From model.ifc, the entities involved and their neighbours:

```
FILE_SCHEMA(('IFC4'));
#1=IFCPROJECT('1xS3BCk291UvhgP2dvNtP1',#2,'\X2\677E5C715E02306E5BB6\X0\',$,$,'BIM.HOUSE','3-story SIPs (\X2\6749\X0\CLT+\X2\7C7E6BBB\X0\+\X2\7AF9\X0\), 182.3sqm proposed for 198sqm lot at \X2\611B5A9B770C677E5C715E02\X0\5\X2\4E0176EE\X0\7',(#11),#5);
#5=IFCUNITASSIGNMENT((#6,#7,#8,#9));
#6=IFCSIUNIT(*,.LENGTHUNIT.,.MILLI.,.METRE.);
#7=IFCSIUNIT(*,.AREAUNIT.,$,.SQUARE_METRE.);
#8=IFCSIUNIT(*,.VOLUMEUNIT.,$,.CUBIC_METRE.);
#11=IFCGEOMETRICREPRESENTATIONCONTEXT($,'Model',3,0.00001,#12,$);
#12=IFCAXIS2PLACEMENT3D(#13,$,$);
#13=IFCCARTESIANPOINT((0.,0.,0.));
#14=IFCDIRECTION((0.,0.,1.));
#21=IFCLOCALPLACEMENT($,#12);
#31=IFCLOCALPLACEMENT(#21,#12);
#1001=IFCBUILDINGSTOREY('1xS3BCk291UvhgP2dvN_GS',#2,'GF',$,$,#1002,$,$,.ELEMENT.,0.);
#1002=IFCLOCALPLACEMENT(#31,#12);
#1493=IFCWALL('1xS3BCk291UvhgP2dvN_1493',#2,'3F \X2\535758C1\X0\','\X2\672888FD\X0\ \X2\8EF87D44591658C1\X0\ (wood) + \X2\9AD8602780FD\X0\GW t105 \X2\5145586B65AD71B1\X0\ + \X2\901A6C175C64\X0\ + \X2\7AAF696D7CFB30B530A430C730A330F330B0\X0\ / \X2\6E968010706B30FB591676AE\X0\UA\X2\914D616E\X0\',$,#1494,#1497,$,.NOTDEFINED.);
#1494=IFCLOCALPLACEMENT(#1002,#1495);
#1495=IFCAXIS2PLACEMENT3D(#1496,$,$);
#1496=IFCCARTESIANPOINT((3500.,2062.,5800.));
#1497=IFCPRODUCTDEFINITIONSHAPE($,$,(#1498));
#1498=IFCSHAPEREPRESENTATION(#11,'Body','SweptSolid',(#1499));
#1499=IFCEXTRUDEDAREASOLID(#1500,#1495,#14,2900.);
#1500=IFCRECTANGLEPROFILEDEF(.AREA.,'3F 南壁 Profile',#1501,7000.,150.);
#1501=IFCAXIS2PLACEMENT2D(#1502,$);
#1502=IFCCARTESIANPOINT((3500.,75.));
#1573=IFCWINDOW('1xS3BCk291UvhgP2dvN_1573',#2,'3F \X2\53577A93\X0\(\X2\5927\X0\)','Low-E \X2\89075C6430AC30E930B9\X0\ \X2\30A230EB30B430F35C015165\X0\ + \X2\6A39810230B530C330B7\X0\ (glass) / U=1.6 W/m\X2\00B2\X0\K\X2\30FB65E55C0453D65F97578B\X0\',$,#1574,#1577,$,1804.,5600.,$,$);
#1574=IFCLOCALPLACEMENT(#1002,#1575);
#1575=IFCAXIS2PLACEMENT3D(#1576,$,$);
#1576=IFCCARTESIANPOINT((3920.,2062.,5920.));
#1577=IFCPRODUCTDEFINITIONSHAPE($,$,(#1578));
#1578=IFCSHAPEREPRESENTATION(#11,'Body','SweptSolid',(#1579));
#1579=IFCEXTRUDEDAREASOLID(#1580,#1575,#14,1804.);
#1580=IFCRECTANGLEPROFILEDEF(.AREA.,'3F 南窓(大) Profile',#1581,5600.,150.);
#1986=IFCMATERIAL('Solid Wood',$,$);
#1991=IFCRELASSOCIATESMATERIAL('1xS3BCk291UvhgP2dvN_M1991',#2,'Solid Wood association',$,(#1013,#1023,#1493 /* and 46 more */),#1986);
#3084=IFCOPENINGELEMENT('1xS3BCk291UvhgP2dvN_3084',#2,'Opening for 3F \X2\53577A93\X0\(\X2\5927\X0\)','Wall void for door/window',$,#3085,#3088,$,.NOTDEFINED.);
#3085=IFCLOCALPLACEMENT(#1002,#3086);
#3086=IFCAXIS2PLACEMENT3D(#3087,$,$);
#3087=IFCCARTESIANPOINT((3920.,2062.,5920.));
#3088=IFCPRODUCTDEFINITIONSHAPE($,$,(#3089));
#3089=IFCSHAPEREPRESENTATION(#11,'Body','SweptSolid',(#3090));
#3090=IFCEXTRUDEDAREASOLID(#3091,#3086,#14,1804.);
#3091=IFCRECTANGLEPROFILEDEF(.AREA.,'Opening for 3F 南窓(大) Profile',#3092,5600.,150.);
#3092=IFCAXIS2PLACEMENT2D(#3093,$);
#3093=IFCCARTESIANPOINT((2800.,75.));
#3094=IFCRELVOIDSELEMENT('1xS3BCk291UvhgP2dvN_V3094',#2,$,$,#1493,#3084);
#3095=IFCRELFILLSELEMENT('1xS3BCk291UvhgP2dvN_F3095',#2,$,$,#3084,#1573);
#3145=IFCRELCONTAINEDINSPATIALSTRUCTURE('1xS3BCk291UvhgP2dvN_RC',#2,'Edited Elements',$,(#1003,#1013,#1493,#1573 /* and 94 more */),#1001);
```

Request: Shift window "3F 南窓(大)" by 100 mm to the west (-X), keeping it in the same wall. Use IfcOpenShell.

```python
import ifcopenshell
import ifcopenshell.api.geometry
import ifcopenshell.util.placement

model = ifcopenshell.open("model.ifc")

window = model.by_guid("1xS3BCk291UvhgP2dvN_1573")
opening = window.FillsVoids[0].RelatingOpeningElement
wall = opening.VoidsElements[0].RelatingBuildingElement

wall_matrix = ifcopenshell.util.placement.get_local_placement(wall.ObjectPlacement)
shift = wall_matrix[:3, 0] * -100.0
before = ifcopenshell.util.placement.get_local_placement(window.ObjectPlacement)[:3, 3].copy()

# The window is not placed relative to its opening, so move both.
for product in (opening, window):
    matrix = ifcopenshell.util.placement.get_local_placement(product.ObjectPlacement)
    matrix[:3, 3] += shift
    ifcopenshell.api.geometry.edit_object_placement(model, product=product, matrix=matrix, is_si=False)

after = ifcopenshell.util.placement.get_local_placement(window.ObjectPlacement)[:3, 3]
print("window moved by", (after - before).round(3) + 0.0)

model.write("model_updated.ifc")
```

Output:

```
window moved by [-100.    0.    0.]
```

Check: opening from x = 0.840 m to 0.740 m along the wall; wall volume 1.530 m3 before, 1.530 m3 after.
